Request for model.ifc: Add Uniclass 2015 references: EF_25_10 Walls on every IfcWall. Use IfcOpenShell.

First a look at what the model holds.

```python
import ifcopenshell

model = ifcopenshell.open("model.ifc")
print(model.schema)
print("classifications:", [c.Name for c in model.by_type("IfcClassification")])
for ifc_class in ("IfcDoor", "IfcRoof", "IfcStair", "IfcWall", "IfcWindow"):
    print(ifc_class, len(model.by_type(ifc_class)))
```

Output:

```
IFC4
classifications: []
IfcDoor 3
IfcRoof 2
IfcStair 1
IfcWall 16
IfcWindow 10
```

```python
import ifcopenshell
import ifcopenshell.api.classification

model = ifcopenshell.open("model.ifc")

system = ifcopenshell.api.classification.add_classification(model, classification="Uniclass 2015")

codes = {
    "IfcWall": ("EF_25_10", "Walls"),
}
for ifc_class, (code, name) in codes.items():
    products = model.by_type(ifc_class)
    ifcopenshell.api.classification.add_reference(
        model, products=products, classification=system, identification=code, name=name
    )
    print(code, len(products))

model.write("model_edited.ifc")
```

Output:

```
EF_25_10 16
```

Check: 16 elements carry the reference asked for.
